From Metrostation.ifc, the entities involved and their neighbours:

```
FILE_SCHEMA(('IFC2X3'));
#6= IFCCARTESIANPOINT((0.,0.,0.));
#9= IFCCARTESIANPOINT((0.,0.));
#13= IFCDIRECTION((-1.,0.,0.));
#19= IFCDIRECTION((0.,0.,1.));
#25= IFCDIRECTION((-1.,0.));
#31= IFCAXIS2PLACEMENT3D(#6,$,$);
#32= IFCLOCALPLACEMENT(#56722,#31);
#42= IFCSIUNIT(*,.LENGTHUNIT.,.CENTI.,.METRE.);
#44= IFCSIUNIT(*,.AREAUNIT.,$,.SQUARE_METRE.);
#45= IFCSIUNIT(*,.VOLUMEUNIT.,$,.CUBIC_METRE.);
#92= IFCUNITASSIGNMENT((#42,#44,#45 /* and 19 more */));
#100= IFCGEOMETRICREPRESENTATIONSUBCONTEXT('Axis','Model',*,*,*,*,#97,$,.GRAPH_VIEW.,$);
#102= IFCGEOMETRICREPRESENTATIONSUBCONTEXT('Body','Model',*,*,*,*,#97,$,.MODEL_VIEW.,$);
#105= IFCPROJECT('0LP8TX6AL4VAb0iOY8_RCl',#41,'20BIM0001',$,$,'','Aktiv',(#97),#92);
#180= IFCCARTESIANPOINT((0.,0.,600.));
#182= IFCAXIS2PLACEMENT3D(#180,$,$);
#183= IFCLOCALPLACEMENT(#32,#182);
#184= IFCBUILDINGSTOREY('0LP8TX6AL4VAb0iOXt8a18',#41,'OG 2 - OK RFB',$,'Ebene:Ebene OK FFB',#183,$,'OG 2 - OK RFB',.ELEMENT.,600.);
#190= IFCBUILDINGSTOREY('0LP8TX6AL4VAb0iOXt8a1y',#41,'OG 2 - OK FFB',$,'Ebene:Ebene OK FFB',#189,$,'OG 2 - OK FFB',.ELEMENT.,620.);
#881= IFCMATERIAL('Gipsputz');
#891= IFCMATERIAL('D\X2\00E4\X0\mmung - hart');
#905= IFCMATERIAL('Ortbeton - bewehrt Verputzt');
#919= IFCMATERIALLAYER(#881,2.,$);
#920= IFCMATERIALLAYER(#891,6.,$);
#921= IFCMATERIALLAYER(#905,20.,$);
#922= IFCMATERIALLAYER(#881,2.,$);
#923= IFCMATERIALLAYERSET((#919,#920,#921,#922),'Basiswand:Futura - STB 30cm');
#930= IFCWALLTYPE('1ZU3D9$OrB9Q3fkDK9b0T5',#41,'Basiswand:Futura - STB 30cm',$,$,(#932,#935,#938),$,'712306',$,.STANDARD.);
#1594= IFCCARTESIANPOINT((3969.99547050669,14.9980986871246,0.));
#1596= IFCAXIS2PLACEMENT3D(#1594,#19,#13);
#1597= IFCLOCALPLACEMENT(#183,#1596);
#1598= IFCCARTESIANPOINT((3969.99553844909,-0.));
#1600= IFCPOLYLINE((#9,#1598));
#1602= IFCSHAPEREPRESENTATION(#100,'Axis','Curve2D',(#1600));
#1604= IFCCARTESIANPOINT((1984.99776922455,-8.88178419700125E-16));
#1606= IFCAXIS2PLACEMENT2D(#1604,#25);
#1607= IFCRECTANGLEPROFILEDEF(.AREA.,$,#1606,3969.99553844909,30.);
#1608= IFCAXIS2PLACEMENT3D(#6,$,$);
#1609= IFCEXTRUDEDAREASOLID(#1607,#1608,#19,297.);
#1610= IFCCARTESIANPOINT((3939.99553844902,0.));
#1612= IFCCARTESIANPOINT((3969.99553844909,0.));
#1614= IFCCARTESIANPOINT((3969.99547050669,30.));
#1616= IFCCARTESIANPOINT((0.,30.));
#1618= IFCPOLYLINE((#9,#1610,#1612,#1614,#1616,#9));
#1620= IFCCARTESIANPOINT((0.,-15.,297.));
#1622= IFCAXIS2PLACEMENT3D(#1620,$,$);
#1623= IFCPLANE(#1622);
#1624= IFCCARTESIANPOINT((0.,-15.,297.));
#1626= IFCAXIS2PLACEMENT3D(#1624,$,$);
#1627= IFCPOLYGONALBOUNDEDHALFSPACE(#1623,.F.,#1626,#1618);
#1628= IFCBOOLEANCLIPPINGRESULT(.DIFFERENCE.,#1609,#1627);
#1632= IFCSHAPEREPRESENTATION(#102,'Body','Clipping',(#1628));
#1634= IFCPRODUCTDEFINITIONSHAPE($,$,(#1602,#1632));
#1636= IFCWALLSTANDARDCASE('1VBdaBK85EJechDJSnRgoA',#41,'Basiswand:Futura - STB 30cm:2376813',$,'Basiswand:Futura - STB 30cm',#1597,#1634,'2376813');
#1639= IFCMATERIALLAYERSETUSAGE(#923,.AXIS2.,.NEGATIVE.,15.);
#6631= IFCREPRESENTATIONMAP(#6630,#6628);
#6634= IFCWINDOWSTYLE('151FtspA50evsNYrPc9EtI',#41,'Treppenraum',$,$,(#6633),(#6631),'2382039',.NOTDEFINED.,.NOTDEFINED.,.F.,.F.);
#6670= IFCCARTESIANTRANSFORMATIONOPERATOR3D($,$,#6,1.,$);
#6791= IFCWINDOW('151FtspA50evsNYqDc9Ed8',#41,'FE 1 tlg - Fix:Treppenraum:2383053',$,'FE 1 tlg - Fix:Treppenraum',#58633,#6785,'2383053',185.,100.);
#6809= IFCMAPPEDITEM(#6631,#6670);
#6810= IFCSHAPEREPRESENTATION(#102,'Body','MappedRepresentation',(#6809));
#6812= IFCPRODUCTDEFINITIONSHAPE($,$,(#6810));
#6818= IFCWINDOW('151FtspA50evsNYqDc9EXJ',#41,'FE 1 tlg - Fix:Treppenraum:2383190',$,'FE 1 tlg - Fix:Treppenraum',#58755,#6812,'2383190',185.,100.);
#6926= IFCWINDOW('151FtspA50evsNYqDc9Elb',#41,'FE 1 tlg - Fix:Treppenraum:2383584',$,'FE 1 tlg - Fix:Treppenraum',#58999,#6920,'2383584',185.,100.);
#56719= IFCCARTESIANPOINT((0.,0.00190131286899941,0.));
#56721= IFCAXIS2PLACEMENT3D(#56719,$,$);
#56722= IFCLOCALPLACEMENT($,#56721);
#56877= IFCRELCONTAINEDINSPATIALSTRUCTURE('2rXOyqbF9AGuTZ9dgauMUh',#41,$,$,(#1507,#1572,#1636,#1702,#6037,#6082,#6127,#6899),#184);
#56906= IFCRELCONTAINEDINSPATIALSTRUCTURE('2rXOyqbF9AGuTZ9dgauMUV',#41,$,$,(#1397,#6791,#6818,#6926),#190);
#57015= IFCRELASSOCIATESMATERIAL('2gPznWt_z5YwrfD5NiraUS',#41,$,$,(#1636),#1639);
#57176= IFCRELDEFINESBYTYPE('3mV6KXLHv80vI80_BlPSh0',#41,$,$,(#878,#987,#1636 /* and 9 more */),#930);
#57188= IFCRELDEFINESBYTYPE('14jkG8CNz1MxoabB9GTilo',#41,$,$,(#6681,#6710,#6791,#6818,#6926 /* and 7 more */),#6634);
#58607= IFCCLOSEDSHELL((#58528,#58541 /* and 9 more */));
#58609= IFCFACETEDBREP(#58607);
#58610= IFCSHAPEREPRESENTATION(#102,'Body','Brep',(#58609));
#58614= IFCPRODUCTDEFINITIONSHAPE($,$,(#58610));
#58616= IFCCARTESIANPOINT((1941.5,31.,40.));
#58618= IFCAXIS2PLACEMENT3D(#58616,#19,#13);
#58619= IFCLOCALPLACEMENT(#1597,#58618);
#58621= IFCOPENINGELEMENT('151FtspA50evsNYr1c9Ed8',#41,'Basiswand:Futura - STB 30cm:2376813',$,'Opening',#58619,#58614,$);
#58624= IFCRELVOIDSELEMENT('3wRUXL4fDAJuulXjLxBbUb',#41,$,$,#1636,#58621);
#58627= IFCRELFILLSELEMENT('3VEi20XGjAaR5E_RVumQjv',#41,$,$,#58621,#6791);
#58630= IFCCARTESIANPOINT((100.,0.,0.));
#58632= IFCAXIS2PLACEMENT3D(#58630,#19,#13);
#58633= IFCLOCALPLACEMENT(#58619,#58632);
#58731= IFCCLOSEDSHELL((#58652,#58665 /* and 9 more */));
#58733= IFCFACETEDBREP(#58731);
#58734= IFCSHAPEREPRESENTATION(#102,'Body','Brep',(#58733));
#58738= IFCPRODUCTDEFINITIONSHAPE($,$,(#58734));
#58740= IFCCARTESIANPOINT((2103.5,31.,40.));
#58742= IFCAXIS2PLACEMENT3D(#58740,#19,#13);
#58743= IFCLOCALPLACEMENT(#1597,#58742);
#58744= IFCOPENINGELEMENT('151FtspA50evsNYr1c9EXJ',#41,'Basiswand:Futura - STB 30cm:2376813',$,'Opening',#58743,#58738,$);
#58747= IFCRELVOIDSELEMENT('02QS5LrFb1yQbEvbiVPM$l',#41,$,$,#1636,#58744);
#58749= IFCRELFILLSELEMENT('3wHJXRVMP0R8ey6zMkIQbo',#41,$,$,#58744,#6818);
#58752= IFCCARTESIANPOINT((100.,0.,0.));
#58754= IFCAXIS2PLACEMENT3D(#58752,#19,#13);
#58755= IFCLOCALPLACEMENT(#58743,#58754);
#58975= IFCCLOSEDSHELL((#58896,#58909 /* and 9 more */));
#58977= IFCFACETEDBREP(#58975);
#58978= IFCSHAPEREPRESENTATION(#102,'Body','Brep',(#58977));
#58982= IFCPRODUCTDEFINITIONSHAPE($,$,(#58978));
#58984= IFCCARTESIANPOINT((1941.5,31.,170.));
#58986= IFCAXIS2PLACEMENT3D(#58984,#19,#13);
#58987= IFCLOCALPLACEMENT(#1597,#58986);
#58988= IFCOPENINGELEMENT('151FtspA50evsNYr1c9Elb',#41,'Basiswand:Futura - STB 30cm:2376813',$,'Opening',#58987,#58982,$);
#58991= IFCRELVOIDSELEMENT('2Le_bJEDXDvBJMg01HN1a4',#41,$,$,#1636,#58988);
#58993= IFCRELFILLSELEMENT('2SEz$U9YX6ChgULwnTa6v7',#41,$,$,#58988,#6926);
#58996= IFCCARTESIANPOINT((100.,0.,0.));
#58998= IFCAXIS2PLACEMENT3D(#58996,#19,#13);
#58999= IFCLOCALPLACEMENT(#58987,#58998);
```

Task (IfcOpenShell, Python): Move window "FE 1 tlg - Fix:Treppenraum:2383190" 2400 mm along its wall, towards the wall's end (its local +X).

```python
import ifcopenshell
import ifcopenshell.api.geometry
import ifcopenshell.util.placement
import ifcopenshell.util.unit

model = ifcopenshell.open("Metrostation.ifc")
unit_scale = ifcopenshell.util.unit.calculate_unit_scale(model)

window = model.by_guid("151FtspA50evsNYqDc9EXJ")
opening = window.FillsVoids[0].RelatingOpeningElement
wall = opening.VoidsElements[0].RelatingBuildingElement

wall_matrix = ifcopenshell.util.placement.get_local_placement(wall.ObjectPlacement)
shift = wall_matrix[:3, 0] * 2.4 / unit_scale
before = ifcopenshell.util.placement.get_local_placement(window.ObjectPlacement)[:3, 3].copy()

# The window is placed relative to its opening, so it follows when the opening moves.
matrix = ifcopenshell.util.placement.get_local_placement(opening.ObjectPlacement)
matrix[:3, 3] += shift
ifcopenshell.api.geometry.edit_object_placement(
    model, product=opening, matrix=matrix, is_si=False, should_transform_children=True
)

after = ifcopenshell.util.placement.get_local_placement(window.ObjectPlacement)[:3, 3]
print("window moved by", (after - before).round(3) + 0.0)

model.write("Metrostation_v2.ifc")
```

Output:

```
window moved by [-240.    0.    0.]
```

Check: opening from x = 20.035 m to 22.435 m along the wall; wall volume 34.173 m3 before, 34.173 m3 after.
